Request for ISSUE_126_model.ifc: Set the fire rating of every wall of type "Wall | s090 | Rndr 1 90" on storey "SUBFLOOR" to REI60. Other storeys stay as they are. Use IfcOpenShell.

First a look at what the model holds.

```python
import ifcopenshell
import ifcopenshell.util.element

model = ifcopenshell.open("ISSUE_126_model.ifc")
print(model.schema)
storey = next(s for s in model.by_type("IfcBuildingStorey") if s.Name == "SUBFLOOR")
walls = [e for e in ifcopenshell.util.element.get_decomposition(storey) if e.is_a("IfcWall")]
seen = {}
for e in walls:
    element_type = ifcopenshell.util.element.get_type(e)
    key = (element_type.Name if element_type != e and element_type else None, ifcopenshell.util.element.get_pset(e, "Pset_WallCommon", "FireRating"))
    seen[key] = seen.get(key, 0) + 1
for (name, value), count in sorted(seen.items(), key=str):
    print(count, "x", name, "|", value)
```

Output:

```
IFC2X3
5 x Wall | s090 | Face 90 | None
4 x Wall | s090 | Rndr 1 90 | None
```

```python
import ifcopenshell
import ifcopenshell.api.pset
import ifcopenshell.util.element

model = ifcopenshell.open("ISSUE_126_model.ifc")

storey = next(s for s in model.by_type("IfcBuildingStorey") if s.Name == "SUBFLOOR")
walls = [e for e in ifcopenshell.util.element.get_decomposition(storey) if e.is_a("IfcWall")]

count = 0
for e in walls:
    element_type = ifcopenshell.util.element.get_type(e)
    if element_type in (None, e) or element_type.Name != "Wall | s090 | Rndr 1 90":
        continue
    # add_pset returns the element's existing set when there is one.
    pset = ifcopenshell.api.pset.add_pset(model, product=e, name="Pset_WallCommon")
    ifcopenshell.api.pset.edit_pset(model, pset=pset, properties={"FireRating": "REI60"})
    count += 1

print(count, "walls updated")

model.write("ISSUE_126_model_rev.ifc")
```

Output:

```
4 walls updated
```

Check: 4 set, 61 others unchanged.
